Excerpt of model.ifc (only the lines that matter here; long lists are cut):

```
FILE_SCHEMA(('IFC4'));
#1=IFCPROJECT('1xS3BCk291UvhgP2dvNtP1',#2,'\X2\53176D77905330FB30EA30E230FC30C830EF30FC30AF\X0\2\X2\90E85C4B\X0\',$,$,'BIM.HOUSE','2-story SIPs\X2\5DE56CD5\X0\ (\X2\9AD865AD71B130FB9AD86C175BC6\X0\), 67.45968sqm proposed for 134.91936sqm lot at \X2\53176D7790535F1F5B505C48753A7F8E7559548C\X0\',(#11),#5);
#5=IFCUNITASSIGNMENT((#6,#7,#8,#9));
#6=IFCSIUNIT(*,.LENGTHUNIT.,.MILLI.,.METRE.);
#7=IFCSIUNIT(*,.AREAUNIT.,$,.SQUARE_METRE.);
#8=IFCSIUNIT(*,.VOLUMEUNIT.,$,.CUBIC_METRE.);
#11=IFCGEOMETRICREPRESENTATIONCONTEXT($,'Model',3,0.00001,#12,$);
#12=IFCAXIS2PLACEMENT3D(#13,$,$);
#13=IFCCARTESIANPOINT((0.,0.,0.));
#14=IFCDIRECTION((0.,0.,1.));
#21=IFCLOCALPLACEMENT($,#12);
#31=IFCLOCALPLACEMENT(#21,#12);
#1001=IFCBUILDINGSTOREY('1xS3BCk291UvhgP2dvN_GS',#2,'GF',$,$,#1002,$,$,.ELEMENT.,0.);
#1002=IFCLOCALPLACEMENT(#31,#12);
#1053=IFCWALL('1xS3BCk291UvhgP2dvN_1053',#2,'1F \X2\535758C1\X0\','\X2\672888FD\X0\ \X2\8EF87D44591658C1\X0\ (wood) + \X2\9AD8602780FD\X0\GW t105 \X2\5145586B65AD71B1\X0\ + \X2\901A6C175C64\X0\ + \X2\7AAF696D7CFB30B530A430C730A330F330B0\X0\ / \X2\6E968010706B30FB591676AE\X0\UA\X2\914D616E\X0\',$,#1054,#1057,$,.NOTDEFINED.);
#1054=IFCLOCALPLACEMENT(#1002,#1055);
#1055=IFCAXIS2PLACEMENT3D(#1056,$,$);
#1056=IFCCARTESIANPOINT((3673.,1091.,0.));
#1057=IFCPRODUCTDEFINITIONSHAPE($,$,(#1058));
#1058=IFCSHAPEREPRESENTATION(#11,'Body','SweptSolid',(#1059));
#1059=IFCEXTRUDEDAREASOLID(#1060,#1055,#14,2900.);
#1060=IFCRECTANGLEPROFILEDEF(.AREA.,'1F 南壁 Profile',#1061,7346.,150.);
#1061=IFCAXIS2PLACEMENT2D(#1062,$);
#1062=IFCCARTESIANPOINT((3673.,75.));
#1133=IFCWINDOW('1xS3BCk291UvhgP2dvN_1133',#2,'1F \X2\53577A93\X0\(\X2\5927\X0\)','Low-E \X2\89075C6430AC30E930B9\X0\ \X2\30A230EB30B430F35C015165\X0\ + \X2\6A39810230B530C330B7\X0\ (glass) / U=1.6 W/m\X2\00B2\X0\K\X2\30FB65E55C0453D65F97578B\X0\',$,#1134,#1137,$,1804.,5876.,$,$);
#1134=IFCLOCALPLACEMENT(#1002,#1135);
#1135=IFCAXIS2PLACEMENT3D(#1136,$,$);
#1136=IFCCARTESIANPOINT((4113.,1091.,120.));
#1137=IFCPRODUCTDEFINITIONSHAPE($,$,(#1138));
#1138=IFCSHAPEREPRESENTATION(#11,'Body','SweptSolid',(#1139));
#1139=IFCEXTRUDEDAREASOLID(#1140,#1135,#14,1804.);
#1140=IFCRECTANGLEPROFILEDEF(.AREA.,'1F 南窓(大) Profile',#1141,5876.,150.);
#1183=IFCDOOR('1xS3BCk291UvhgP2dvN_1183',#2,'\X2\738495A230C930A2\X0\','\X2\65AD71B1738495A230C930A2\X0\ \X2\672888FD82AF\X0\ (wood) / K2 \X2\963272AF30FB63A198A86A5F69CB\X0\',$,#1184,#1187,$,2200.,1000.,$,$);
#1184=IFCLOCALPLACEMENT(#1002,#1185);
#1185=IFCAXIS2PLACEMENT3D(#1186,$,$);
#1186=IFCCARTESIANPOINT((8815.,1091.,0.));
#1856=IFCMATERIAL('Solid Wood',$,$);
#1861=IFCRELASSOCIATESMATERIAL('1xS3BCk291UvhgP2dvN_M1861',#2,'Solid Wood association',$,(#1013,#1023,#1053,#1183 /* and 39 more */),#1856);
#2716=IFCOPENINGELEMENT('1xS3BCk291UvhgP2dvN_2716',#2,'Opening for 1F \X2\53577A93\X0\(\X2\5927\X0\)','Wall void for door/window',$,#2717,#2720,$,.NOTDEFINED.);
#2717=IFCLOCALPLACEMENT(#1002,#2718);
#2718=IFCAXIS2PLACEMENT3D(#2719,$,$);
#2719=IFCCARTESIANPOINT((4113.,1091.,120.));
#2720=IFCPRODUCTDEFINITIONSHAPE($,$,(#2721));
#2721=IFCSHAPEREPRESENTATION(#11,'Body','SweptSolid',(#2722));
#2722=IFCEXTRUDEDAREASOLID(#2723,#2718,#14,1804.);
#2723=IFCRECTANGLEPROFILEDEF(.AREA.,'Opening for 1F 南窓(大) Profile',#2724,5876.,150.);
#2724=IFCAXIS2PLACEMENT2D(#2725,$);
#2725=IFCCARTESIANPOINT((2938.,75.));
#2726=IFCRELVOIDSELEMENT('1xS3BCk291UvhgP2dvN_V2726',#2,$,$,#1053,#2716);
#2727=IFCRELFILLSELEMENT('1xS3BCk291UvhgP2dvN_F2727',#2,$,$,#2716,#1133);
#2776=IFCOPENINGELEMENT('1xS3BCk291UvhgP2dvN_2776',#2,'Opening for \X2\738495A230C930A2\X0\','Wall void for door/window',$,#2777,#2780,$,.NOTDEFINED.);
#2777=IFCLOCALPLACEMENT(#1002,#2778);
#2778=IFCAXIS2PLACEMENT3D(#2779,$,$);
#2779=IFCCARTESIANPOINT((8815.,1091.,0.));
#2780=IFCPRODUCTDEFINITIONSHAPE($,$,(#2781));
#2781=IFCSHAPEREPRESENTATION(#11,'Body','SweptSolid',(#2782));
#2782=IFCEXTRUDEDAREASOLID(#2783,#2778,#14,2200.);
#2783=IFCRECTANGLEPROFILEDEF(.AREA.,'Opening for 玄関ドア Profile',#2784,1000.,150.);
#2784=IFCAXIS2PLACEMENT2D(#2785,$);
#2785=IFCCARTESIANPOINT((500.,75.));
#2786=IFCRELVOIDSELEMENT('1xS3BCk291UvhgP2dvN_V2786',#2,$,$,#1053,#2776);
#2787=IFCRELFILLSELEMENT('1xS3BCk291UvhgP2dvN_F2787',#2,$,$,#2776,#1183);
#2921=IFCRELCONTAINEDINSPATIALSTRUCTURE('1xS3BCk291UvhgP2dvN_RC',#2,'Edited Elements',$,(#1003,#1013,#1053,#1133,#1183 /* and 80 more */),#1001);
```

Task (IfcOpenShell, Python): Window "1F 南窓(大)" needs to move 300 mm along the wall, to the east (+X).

```python
import ifcopenshell
import ifcopenshell.api.geometry
import ifcopenshell.util.placement

model = ifcopenshell.open("model.ifc")

window = model.by_guid("1xS3BCk291UvhgP2dvN_1133")
opening = window.FillsVoids[0].RelatingOpeningElement
wall = opening.VoidsElements[0].RelatingBuildingElement

wall_matrix = ifcopenshell.util.placement.get_local_placement(wall.ObjectPlacement)
shift = wall_matrix[:3, 0] * 300.0
before = ifcopenshell.util.placement.get_local_placement(window.ObjectPlacement)[:3, 3].copy()

# The window is not placed relative to its opening, so move both.
for product in (opening, window):
    matrix = ifcopenshell.util.placement.get_local_placement(product.ObjectPlacement)
    matrix[:3, 3] += shift
    ifcopenshell.api.geometry.edit_object_placement(model, product=product, matrix=matrix, is_si=False)

after = ifcopenshell.util.placement.get_local_placement(window.ObjectPlacement)[:3, 3]
print("window moved by", (after - before).round(3) + 0.0)

model.write("model_v2.ifc")
```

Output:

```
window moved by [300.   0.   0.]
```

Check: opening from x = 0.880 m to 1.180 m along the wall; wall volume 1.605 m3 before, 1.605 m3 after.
